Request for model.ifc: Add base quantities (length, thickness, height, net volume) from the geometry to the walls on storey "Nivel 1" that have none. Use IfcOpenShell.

First a look at what the model holds.

```python
import ifcopenshell
import ifcopenshell.util.element
import ifcopenshell.util.unit

model = ifcopenshell.open("model.ifc")
print(model.schema)
for unit_type in ("LENGTHUNIT", "AREAUNIT", "VOLUMEUNIT"):
    print(unit_type, ifcopenshell.util.unit.calculate_unit_scale(model, unit_type))
storey = next(s for s in model.by_type("IfcBuildingStorey") if s.Name == "Nivel 1")
walls = [e for e in ifcopenshell.util.element.get_decomposition(storey) if e.is_a("IfcWall")]
for e in sorted(walls, key=lambda e: e.id()):
    print(e.id(), e.is_a(), e.Name, list(ifcopenshell.util.element.get_psets(e, qtos_only=True)), sep=" | ")
```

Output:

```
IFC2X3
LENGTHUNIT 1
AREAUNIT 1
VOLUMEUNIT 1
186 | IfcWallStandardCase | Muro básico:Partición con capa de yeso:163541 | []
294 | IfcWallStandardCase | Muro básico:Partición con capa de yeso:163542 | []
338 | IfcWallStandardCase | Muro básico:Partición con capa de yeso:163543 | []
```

```python
import ifcopenshell
import ifcopenshell.api.pset
import ifcopenshell.geom
import ifcopenshell.util.element
import ifcopenshell.util.shape
import ifcopenshell.util.unit

model = ifcopenshell.open("model.ifc")
unit_scale = ifcopenshell.util.unit.calculate_unit_scale(model)
volume_scale = ifcopenshell.util.unit.calculate_unit_scale(model, "VOLUMEUNIT")
settings = ifcopenshell.geom.settings()

storey = next(s for s in model.by_type("IfcBuildingStorey") if s.Name == "Nivel 1")
walls = [e for e in ifcopenshell.util.element.get_decomposition(storey) if e.is_a("IfcWall")]

for e in sorted(walls, key=lambda e: e.id()):
    if ifcopenshell.util.element.get_psets(e, qtos_only=True, should_inherit=False):
        continue
    # Geometry comes back in metres, in the element's own axes.
    shape = ifcopenshell.geom.create_shape(settings, e)
    values = {
        "Length": ifcopenshell.util.shape.get_x(shape.geometry) / unit_scale,
        "Width": ifcopenshell.util.shape.get_y(shape.geometry) / unit_scale,
        "Height": ifcopenshell.util.shape.get_z(shape.geometry) / unit_scale,
        "NetVolume": ifcopenshell.util.shape.get_volume(shape.geometry) / volume_scale,
    }
    qto = ifcopenshell.api.pset.add_qto(model, product=e, name="BaseQuantities")
    ifcopenshell.api.pset.edit_qto(model, qto=qto, properties=values)
    print(e.id(), {k: round(v, 3) for k, v in values.items()})

model.write("model_updated.ifc")
```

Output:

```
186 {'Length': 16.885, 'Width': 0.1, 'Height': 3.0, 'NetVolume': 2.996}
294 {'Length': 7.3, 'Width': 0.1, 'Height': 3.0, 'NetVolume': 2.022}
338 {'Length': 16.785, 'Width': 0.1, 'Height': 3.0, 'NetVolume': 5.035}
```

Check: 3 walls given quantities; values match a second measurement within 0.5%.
